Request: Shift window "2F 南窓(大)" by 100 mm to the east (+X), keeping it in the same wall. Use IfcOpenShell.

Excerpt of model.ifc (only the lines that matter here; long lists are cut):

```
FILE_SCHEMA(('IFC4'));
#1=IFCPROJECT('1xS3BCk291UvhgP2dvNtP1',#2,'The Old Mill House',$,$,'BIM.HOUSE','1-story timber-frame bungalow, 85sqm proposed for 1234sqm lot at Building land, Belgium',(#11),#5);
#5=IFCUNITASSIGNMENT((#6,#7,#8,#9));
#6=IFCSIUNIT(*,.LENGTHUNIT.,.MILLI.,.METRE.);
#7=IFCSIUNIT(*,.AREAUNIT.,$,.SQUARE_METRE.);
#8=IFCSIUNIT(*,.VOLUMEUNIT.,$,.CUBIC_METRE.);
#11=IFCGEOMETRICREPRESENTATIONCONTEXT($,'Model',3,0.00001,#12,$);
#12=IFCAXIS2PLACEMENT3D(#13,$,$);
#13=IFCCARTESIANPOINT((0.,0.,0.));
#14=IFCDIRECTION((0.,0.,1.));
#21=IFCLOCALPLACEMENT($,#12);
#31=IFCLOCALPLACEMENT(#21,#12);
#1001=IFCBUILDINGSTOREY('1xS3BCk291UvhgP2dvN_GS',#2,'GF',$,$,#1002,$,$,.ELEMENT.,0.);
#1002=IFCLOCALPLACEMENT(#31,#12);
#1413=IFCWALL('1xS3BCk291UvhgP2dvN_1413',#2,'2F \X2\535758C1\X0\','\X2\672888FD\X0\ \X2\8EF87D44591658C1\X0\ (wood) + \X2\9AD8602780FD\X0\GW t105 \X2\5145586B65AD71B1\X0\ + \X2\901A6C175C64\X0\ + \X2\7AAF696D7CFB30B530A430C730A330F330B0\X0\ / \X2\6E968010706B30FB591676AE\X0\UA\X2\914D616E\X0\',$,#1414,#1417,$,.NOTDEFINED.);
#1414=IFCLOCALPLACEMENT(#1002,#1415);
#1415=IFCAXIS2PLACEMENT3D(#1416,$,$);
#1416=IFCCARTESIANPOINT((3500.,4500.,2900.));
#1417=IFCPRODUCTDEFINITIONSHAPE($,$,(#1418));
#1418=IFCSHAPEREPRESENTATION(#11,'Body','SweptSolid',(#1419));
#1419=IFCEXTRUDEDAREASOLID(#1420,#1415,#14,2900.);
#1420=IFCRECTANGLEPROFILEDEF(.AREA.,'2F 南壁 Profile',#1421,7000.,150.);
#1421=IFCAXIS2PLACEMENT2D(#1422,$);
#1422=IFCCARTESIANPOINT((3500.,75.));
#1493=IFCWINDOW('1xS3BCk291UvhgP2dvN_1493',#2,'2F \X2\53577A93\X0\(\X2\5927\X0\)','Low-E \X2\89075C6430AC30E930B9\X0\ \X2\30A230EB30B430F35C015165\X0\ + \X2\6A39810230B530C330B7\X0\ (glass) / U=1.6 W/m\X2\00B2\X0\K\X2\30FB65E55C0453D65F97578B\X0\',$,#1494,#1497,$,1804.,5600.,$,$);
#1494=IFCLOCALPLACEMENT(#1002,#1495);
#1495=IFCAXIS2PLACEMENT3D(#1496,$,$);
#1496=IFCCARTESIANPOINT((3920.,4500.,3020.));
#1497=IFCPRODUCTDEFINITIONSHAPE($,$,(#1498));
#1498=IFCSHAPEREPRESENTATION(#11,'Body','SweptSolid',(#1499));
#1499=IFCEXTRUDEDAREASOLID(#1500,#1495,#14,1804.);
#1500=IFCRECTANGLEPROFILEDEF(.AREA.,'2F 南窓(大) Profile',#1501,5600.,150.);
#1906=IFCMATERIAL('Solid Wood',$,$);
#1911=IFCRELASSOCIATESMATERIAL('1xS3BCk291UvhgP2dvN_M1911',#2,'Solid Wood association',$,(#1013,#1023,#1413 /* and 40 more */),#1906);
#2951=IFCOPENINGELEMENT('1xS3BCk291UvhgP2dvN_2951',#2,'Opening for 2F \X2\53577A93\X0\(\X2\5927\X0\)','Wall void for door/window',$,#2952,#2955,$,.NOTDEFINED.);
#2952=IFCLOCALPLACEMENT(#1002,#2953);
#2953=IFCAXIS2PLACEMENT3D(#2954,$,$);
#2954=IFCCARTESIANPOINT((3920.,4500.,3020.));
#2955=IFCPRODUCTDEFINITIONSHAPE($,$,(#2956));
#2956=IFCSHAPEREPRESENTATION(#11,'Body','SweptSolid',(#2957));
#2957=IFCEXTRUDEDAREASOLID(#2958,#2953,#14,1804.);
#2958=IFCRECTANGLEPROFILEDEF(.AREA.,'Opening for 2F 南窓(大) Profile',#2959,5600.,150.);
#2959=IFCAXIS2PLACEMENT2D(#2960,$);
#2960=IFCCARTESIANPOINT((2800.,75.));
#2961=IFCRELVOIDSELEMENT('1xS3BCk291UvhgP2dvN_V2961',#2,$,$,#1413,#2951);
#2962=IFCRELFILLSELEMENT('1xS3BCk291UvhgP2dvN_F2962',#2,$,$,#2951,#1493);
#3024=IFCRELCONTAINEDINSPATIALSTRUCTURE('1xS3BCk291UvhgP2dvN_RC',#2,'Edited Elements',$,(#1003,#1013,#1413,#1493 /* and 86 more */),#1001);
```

```python
import ifcopenshell
import ifcopenshell.api.geometry
import ifcopenshell.util.placement
import ifcopenshell.util.unit

model = ifcopenshell.open("model.ifc")
unit_scale = ifcopenshell.util.unit.calculate_unit_scale(model)

window = model.by_id(1493)
opening = window.FillsVoids[0].RelatingOpeningElement
wall = opening.VoidsElements[0].RelatingBuildingElement

wall_matrix = ifcopenshell.util.placement.get_local_placement(wall.ObjectPlacement)
shift = wall_matrix[:3, 0] * 0.1 / unit_scale
before = ifcopenshell.util.placement.get_local_placement(window.ObjectPlacement)[:3, 3].copy()

# The window is not placed relative to its opening, so move both.
for product in (opening, window):
    matrix = ifcopenshell.util.placement.get_local_placement(product.ObjectPlacement)
    matrix[:3, 3] += shift
    ifcopenshell.api.geometry.edit_object_placement(model, product=product, matrix=matrix, is_si=False)

after = ifcopenshell.util.placement.get_local_placement(window.ObjectPlacement)[:3, 3]
print("window moved by", (after - before).round(3) + 0.0)

model.write("model_rev.ifc")
```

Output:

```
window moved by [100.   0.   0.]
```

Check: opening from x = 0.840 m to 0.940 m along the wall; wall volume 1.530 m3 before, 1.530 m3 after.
